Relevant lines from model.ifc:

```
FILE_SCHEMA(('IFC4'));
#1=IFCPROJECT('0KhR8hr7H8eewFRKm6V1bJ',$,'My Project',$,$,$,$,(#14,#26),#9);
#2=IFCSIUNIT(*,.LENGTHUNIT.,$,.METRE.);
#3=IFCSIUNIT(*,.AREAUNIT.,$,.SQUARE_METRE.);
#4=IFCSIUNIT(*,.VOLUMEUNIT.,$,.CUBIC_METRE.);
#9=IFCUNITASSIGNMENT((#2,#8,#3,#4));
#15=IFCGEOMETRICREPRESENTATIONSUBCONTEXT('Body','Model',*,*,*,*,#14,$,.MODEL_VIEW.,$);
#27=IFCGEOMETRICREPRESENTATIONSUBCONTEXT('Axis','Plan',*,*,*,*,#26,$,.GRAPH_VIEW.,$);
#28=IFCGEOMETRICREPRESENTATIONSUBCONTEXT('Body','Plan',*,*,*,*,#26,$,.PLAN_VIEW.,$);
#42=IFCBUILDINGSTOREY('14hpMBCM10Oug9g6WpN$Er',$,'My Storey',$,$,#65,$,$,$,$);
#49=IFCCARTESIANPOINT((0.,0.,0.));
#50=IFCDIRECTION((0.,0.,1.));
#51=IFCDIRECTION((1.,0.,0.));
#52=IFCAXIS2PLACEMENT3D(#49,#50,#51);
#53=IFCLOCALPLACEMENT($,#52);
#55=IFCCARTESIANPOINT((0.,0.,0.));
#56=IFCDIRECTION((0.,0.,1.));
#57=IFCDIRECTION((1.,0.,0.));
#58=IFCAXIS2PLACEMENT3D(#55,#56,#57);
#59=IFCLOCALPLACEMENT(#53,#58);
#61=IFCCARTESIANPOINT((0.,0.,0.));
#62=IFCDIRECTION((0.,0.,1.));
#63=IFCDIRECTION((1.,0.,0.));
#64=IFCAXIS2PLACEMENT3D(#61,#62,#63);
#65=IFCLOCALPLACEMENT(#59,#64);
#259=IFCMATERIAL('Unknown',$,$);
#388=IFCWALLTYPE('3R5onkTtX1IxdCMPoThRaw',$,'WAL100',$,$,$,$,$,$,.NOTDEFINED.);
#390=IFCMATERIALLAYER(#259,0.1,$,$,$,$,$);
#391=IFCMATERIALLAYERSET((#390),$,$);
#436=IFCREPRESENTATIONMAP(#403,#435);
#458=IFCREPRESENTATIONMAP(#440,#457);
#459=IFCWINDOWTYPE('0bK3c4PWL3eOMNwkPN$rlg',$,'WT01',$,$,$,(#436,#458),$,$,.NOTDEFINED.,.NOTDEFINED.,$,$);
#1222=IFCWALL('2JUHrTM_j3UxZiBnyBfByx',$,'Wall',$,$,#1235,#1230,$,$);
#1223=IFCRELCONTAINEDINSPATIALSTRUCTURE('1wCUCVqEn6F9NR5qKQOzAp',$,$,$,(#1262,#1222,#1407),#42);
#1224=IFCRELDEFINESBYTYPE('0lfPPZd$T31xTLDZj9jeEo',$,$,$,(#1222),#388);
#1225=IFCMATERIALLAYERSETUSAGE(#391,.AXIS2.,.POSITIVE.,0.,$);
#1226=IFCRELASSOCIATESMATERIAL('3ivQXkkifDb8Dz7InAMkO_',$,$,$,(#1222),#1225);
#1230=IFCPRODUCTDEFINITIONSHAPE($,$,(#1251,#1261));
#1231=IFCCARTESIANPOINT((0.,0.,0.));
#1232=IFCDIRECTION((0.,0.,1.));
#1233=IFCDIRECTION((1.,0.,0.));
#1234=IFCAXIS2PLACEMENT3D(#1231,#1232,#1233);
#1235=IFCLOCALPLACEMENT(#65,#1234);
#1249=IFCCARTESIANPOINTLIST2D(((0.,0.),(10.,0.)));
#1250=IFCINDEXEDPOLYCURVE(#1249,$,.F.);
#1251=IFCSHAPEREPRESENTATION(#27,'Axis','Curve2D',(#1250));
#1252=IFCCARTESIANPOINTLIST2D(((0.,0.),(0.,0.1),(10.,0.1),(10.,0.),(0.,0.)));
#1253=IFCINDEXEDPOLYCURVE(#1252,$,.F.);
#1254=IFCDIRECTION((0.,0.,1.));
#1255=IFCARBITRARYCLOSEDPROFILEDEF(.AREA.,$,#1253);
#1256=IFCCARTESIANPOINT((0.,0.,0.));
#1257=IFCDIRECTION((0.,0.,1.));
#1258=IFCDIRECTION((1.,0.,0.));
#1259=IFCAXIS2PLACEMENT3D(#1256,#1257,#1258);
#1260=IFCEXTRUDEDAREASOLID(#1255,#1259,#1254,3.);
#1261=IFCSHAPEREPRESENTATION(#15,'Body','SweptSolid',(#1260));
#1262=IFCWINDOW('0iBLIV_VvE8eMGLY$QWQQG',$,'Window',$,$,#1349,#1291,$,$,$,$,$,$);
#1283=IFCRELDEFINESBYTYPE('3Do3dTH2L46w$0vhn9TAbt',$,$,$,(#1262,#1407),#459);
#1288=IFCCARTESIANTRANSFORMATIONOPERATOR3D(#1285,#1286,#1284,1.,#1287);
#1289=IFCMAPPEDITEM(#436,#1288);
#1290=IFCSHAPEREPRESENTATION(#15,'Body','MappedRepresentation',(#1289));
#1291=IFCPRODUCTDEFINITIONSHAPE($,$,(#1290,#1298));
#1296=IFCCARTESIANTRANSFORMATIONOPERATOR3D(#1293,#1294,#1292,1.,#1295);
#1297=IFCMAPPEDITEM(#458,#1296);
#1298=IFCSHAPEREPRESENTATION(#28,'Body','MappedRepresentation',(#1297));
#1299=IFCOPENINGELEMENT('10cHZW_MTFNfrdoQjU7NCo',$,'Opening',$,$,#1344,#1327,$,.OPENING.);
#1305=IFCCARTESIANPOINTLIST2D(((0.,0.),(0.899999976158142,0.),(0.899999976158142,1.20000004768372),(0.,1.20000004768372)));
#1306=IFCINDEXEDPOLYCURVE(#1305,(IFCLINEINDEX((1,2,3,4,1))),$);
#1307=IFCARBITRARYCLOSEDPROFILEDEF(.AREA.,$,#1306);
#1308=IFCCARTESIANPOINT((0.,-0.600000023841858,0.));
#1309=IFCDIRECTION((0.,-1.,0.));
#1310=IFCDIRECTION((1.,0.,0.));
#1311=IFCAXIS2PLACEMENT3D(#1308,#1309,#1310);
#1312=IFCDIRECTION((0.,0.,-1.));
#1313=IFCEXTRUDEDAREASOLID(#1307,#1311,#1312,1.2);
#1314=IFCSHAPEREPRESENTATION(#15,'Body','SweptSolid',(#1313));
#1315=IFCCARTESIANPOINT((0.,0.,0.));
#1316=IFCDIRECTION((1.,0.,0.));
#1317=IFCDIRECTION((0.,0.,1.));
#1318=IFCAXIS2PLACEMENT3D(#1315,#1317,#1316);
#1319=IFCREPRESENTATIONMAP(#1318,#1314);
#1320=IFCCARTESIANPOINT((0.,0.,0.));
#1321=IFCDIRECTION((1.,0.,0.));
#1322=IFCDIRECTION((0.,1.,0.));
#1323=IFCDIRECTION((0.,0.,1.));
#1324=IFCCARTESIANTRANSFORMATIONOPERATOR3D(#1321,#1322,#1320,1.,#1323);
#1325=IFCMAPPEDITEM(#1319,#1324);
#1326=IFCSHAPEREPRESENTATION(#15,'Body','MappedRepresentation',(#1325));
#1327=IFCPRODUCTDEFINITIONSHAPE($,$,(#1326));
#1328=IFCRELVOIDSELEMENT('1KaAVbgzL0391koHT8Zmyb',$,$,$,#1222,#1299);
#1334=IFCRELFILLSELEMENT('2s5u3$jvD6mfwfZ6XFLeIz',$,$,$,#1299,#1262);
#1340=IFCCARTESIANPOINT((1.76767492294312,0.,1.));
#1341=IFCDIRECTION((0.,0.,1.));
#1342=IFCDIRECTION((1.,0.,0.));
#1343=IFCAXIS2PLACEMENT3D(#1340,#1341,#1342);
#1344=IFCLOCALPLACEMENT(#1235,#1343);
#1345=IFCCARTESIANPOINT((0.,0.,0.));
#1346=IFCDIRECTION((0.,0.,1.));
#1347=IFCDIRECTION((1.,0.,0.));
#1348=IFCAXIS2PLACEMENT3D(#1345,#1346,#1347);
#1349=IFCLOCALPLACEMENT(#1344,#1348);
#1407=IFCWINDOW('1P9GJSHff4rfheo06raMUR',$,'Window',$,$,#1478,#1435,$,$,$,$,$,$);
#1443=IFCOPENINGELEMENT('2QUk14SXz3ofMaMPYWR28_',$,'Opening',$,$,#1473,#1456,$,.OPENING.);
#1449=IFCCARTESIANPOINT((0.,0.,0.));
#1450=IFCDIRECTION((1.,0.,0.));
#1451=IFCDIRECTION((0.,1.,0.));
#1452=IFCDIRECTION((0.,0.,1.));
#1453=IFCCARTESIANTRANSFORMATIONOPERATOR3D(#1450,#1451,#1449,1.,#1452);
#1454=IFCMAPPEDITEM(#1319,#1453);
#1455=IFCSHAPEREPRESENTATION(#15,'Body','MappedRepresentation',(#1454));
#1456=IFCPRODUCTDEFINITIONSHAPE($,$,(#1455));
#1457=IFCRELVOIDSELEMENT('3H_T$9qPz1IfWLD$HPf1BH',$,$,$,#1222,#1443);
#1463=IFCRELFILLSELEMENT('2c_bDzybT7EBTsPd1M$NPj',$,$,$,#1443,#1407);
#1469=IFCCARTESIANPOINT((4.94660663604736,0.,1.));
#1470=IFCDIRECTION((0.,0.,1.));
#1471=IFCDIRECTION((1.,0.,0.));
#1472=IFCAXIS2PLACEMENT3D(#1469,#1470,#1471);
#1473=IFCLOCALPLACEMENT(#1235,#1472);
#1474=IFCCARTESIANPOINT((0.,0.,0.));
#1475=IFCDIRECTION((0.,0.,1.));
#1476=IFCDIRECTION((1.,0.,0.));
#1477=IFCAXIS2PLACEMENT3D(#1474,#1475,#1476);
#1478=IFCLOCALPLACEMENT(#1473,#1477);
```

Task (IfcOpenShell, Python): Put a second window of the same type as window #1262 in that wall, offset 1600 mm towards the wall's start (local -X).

```python
import ifcopenshell
import ifcopenshell.api.feature
import ifcopenshell.api.geometry
import ifcopenshell.api.root
import ifcopenshell.geom
import ifcopenshell.util.element
import ifcopenshell.util.placement
import ifcopenshell.util.shape
import ifcopenshell.util.unit

model = ifcopenshell.open("model.ifc")
unit_scale = ifcopenshell.util.unit.calculate_unit_scale(model)
settings = ifcopenshell.geom.settings()


def volume(element):
    """Net volume in cubic metres, openings subtracted."""
    shape = ifcopenshell.geom.create_shape(settings, element)
    return ifcopenshell.util.shape.get_volume(shape.geometry)


window = model.by_id(1262)
opening = window.FillsVoids[0].RelatingOpeningElement
wall = opening.VoidsElements[0].RelatingBuildingElement
before = volume(wall)
shift = ifcopenshell.util.placement.get_local_placement(wall.ObjectPlacement)[:3, 0] * -1.6 / unit_scale

# copy_class copies the void relationship, type, container and properties, but no geometry.
new_opening = ifcopenshell.api.root.copy_class(model, product=opening)
new_opening.Representation = ifcopenshell.util.element.copy_deep(
    model, opening.Representation, exclude=["IfcGeometricRepresentationContext", "IfcRepresentationMap"]
)
new_window = ifcopenshell.api.root.copy_class(model, product=window)
new_window.Representation = ifcopenshell.util.element.copy_deep(
    model, window.Representation, exclude=["IfcGeometricRepresentationContext", "IfcRepresentationMap"]
)
ifcopenshell.api.feature.add_filling(model, opening=new_opening, element=new_window)

for old, new in ((opening, new_opening), (window, new_window)):
    matrix = ifcopenshell.util.placement.get_local_placement(old.ObjectPlacement)
    matrix[:3, 3] += shift
    ifcopenshell.api.geometry.edit_object_placement(model, product=new, matrix=matrix, is_si=False)

after = volume(wall)

print(f"wall volume {before:.3f} -> {after:.3f} m3")

model.write("model-out.ifc")
```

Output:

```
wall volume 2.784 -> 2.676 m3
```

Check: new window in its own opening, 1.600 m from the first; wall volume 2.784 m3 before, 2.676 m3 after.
